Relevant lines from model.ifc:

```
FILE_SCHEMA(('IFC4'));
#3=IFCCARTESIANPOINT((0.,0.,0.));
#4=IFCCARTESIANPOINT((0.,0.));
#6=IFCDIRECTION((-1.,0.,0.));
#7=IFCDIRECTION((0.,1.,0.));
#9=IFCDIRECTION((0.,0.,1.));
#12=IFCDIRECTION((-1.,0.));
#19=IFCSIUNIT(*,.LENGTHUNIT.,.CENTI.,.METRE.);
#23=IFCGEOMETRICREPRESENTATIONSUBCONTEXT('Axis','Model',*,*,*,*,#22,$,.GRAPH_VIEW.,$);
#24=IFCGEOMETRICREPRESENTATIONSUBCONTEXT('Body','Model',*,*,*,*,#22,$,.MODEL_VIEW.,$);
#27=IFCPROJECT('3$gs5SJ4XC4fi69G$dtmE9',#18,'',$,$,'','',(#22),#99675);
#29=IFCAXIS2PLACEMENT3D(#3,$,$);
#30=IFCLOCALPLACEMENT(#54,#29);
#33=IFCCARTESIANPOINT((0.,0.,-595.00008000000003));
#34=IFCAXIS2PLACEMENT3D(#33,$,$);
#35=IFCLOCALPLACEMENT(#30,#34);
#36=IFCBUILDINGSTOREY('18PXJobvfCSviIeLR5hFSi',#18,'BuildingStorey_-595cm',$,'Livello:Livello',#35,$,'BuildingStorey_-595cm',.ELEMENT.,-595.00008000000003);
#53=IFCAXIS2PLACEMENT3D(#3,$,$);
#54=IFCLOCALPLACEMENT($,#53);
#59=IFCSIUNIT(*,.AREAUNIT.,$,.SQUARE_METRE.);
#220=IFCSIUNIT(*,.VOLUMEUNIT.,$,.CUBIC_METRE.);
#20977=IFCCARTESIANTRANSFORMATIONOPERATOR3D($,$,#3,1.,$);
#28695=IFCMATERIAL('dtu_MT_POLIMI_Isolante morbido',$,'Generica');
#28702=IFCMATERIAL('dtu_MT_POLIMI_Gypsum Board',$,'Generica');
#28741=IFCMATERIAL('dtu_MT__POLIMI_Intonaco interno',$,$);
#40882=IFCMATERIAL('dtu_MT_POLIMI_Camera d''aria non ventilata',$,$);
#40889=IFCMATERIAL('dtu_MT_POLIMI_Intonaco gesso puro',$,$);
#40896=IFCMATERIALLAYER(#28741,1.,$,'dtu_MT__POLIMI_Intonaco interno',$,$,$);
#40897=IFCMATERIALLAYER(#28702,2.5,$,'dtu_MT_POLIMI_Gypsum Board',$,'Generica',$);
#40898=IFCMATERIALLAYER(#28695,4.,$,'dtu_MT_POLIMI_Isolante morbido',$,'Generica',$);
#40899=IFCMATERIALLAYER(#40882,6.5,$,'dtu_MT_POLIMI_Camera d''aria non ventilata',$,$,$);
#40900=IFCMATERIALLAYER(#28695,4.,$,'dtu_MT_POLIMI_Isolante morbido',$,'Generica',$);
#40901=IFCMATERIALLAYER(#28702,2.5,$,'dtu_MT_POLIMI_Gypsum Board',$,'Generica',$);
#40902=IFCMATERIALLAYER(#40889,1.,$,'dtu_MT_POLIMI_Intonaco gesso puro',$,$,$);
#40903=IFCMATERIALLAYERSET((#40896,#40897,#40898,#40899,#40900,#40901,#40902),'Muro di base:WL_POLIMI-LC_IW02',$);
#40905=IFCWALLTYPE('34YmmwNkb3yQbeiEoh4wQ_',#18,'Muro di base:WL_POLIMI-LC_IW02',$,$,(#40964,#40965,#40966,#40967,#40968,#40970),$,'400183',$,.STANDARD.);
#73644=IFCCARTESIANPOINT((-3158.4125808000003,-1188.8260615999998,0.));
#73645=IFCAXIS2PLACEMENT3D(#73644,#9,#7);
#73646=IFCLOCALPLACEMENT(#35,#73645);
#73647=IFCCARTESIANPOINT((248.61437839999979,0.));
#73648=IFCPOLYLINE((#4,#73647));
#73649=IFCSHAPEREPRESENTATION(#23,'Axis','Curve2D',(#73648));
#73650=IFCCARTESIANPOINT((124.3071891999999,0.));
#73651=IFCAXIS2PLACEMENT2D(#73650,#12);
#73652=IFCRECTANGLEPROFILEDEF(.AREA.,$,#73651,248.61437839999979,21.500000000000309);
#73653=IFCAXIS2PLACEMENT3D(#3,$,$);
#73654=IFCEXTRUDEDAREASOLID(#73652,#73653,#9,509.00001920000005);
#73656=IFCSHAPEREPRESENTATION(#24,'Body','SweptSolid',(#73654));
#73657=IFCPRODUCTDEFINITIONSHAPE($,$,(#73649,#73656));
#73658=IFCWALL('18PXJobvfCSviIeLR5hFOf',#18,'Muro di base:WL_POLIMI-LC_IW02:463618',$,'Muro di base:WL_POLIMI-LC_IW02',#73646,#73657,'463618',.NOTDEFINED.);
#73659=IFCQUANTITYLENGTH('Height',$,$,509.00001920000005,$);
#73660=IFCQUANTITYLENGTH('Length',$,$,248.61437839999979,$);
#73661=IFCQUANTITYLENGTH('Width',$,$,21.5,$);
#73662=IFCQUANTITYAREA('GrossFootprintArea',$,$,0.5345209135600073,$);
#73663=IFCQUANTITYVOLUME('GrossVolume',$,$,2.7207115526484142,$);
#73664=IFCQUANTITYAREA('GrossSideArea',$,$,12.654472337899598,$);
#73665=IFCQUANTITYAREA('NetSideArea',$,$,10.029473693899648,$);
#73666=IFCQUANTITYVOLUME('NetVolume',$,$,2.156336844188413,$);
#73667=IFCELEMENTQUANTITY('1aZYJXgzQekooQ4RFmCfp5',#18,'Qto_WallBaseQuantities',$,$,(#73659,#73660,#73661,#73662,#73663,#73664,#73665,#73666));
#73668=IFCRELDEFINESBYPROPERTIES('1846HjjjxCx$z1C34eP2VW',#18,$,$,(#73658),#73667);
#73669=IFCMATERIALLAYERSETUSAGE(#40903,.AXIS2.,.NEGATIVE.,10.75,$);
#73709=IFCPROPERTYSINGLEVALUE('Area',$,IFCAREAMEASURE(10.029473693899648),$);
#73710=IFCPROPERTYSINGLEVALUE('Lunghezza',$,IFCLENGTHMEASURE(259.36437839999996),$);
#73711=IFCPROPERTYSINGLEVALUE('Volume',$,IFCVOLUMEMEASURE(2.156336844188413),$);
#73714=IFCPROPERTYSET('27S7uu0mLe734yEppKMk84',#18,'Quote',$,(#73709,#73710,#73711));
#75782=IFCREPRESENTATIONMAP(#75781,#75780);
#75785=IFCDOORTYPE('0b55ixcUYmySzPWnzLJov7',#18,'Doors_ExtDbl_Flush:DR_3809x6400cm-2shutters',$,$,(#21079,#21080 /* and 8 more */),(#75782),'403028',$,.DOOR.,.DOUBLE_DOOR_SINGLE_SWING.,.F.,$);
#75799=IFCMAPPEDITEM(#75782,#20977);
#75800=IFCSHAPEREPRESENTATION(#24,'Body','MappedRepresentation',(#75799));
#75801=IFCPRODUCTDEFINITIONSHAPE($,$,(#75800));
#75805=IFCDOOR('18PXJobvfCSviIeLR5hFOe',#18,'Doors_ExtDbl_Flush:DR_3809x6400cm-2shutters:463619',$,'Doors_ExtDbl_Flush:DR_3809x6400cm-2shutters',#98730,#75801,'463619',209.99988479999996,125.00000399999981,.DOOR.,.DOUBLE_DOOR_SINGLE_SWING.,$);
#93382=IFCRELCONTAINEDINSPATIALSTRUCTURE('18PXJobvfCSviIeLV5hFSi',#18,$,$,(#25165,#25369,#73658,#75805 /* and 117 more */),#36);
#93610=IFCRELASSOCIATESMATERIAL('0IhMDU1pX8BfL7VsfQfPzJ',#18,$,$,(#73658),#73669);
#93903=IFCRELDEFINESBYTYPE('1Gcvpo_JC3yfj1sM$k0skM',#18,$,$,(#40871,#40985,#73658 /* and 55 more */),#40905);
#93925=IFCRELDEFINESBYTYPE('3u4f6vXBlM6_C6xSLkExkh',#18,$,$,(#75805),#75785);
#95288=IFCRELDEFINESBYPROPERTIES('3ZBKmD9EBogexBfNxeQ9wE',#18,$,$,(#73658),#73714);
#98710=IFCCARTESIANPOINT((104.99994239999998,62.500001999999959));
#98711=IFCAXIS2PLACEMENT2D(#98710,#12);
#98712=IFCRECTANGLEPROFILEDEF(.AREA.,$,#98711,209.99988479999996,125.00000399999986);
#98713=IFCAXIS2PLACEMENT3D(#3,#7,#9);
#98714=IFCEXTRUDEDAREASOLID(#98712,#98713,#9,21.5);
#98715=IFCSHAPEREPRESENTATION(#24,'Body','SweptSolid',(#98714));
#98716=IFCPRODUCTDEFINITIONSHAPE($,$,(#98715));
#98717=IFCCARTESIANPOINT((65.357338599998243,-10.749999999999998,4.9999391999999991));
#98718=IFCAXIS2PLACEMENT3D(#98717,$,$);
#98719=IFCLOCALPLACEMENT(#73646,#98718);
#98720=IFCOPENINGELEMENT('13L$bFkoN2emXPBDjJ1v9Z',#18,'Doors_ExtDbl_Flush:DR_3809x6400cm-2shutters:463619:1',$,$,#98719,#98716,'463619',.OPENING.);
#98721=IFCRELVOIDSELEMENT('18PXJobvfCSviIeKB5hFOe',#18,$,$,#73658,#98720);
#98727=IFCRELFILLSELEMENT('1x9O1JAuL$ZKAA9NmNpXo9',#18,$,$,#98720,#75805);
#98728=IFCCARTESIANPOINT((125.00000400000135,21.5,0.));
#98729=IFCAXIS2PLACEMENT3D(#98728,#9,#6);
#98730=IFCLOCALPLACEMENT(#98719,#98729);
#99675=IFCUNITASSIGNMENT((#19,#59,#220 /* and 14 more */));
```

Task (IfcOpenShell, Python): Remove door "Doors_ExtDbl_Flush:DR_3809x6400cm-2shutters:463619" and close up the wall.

```python
import ifcopenshell
import ifcopenshell.api.feature
import ifcopenshell.api.pset
import ifcopenshell.api.root
import ifcopenshell.geom
import ifcopenshell.util.element
import ifcopenshell.util.shape
import ifcopenshell.util.unit

model = ifcopenshell.open("model.ifc")
area_scale = ifcopenshell.util.unit.calculate_unit_scale(model, "AREAUNIT")
volume_scale = ifcopenshell.util.unit.calculate_unit_scale(model, "VOLUMEUNIT")
settings = ifcopenshell.geom.settings()


def volume(element):
    """Net volume in cubic metres, openings subtracted."""
    shape = ifcopenshell.geom.create_shape(settings, element)
    return ifcopenshell.util.shape.get_volume(shape.geometry)


door = model.by_guid("18PXJobvfCSviIeLR5hFOe")
opening = door.FillsVoids[0].RelatingOpeningElement
wall = opening.VoidsElements[0].RelatingBuildingElement
before = volume(wall)

ifcopenshell.api.root.remove_product(model, product=door)
ifcopenshell.api.feature.remove_feature(model, feature=opening)

after = volume(wall)
thickness = 0.215  # wall thickness in metres

# Update the wall's stored quantities.
qto = model.by_id(ifcopenshell.util.element.get_pset(wall, "Qto_WallBaseQuantities", should_inherit=False)["id"])
ifcopenshell.api.pset.edit_qto(model, qto=qto, properties={
    "NetSideArea": after / thickness / area_scale,
    "NetVolume": after / volume_scale,
})
pset = model.by_id(ifcopenshell.util.element.get_pset(wall, "Quote", should_inherit=False)["id"])
ifcopenshell.api.pset.edit_pset(model, pset=pset, properties={
    "Area": model.create_entity("IfcAreaMeasure", after / thickness / area_scale),
    "Volume": model.create_entity("IfcVolumeMeasure", after / volume_scale),
})

print(f"wall volume {before:.3f} -> {after:.3f} m3")

model.write("model-out.ifc")
```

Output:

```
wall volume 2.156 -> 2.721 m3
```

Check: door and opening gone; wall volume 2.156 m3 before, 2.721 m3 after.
